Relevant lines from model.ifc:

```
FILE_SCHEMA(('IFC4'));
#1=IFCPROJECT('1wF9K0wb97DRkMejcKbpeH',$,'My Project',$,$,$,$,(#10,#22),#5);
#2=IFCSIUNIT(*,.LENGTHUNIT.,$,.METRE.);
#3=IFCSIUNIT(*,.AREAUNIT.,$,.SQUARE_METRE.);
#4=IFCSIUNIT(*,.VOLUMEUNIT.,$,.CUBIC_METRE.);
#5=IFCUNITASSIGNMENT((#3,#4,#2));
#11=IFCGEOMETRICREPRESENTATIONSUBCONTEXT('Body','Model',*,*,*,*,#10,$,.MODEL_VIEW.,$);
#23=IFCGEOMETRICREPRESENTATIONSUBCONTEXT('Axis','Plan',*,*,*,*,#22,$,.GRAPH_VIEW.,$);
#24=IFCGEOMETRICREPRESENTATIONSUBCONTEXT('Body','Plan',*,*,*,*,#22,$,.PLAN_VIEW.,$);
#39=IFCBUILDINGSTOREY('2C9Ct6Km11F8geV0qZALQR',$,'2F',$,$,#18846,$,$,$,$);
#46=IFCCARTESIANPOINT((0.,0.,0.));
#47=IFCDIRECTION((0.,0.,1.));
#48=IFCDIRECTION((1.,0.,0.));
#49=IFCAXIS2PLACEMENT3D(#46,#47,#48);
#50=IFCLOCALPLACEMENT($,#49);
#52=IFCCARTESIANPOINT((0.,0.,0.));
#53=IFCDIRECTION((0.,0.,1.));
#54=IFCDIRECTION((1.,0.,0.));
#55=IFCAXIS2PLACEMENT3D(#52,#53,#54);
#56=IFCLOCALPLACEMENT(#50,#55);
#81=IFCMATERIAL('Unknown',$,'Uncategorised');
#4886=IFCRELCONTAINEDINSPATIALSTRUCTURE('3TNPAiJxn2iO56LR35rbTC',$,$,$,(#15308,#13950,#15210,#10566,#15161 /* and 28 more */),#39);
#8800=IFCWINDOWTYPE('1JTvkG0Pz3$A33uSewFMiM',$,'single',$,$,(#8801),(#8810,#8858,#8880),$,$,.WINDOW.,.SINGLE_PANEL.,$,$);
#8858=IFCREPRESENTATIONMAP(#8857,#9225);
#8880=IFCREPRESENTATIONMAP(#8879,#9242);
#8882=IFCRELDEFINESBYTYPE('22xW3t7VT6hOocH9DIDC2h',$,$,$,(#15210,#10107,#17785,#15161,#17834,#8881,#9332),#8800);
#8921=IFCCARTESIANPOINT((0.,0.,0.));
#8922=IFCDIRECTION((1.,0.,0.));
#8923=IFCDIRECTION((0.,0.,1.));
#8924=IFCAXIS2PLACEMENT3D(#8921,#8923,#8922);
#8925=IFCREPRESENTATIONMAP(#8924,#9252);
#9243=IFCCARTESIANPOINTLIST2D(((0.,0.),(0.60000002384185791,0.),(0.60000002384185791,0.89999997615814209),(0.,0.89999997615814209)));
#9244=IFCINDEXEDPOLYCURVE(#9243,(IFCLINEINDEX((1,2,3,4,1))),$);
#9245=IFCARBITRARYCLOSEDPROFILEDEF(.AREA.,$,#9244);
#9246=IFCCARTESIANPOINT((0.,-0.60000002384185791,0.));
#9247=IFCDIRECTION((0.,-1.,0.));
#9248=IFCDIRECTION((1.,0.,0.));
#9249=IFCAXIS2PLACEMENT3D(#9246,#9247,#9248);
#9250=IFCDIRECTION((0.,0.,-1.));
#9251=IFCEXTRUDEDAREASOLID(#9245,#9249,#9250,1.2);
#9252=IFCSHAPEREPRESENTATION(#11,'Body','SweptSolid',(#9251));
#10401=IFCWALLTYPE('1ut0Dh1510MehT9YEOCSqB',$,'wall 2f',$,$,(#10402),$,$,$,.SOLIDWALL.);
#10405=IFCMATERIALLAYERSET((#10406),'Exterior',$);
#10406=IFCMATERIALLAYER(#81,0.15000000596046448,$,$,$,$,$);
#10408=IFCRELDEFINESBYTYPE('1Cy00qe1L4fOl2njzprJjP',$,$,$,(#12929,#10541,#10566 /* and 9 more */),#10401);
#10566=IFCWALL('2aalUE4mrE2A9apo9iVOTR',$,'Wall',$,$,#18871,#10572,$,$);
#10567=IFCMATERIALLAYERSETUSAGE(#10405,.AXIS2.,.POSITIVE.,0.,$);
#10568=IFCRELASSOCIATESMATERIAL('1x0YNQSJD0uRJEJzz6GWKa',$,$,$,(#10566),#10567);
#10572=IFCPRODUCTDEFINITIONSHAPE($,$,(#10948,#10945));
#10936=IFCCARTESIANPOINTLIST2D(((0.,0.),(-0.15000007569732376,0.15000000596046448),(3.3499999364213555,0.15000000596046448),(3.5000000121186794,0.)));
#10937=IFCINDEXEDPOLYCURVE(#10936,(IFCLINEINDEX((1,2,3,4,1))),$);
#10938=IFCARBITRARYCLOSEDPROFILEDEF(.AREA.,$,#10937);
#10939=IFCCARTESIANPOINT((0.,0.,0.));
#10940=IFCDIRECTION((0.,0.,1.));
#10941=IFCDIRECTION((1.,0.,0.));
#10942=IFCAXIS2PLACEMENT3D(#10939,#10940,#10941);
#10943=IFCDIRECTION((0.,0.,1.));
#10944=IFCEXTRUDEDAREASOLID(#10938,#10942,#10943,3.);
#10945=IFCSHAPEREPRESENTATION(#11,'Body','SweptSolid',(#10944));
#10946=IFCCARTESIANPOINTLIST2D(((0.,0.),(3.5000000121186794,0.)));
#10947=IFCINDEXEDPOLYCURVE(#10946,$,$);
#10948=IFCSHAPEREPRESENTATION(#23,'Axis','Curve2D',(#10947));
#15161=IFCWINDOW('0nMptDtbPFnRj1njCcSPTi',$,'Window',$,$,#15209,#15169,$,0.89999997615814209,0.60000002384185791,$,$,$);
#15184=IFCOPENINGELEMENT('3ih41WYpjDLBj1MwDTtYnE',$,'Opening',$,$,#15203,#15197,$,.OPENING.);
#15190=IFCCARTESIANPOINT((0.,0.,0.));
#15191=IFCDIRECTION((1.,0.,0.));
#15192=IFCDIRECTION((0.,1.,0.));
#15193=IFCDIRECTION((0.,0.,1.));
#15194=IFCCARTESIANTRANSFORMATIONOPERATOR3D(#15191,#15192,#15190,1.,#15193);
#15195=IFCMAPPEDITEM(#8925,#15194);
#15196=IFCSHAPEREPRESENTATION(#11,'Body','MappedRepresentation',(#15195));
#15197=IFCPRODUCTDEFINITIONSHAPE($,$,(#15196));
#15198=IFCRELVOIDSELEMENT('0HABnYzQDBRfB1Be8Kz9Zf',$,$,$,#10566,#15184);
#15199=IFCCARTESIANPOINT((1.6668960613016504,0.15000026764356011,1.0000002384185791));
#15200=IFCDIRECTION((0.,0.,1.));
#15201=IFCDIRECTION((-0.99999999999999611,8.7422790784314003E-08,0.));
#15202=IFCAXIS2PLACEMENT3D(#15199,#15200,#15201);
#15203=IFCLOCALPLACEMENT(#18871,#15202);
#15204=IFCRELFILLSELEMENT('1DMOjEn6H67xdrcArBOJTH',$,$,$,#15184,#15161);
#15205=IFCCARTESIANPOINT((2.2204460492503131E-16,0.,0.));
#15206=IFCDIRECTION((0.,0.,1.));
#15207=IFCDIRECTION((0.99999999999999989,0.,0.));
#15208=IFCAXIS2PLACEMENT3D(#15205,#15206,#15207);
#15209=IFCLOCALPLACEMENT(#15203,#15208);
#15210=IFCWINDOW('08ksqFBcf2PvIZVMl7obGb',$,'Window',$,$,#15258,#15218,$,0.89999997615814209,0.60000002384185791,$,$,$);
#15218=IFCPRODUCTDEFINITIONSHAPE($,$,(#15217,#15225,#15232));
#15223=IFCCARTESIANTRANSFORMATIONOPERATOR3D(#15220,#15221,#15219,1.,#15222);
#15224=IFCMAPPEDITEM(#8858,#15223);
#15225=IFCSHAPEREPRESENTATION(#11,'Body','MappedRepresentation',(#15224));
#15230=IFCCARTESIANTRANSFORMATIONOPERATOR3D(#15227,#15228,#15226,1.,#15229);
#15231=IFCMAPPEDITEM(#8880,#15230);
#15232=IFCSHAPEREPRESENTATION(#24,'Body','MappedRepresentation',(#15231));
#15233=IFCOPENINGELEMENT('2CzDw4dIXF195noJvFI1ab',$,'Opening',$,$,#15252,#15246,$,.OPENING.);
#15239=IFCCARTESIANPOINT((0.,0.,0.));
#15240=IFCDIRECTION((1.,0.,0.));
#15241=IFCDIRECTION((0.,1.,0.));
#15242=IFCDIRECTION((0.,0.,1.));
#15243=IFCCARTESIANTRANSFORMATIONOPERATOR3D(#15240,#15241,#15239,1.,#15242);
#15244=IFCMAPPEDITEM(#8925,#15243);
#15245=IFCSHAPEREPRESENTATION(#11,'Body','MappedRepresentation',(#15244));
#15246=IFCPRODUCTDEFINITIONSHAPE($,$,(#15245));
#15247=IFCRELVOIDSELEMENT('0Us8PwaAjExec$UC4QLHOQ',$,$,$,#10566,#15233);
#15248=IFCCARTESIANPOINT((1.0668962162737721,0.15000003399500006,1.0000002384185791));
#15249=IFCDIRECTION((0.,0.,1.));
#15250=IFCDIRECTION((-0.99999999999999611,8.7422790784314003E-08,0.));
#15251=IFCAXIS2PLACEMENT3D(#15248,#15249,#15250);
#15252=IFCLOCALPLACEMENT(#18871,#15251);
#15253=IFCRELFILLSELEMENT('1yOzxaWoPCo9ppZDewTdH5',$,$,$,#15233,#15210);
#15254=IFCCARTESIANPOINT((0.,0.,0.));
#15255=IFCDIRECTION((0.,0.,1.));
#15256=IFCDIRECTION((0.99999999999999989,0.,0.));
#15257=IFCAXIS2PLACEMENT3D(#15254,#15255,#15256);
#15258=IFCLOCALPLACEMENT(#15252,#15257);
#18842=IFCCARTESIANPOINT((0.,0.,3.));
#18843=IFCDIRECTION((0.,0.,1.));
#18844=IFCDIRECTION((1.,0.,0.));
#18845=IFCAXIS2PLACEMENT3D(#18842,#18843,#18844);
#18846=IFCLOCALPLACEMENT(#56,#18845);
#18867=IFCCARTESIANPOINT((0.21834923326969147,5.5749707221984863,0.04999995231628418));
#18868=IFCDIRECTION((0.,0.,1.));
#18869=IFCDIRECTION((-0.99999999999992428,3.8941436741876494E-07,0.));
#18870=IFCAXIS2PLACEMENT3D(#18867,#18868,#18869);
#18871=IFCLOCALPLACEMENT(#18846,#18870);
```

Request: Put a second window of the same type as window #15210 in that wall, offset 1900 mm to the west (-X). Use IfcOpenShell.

```python
import ifcopenshell
import ifcopenshell.api.feature
import ifcopenshell.api.geometry
import ifcopenshell.api.root
import ifcopenshell.geom
import ifcopenshell.util.element
import ifcopenshell.util.placement
import ifcopenshell.util.shape
import ifcopenshell.util.unit

model = ifcopenshell.open("model.ifc")
unit_scale = ifcopenshell.util.unit.calculate_unit_scale(model)
settings = ifcopenshell.geom.settings()


def volume(element):
    """Net volume in cubic metres, openings subtracted."""
    shape = ifcopenshell.geom.create_shape(settings, element)
    return ifcopenshell.util.shape.get_volume(shape.geometry)


window = model.by_guid("08ksqFBcf2PvIZVMl7obGb")
opening = window.FillsVoids[0].RelatingOpeningElement
wall = opening.VoidsElements[0].RelatingBuildingElement
before = volume(wall)
shift = ifcopenshell.util.placement.get_local_placement(wall.ObjectPlacement)[:3, 0] * 1.9 / unit_scale

# copy_class copies the void relationship, type, container and properties, but no geometry.
new_opening = ifcopenshell.api.root.copy_class(model, product=opening)
new_opening.Representation = ifcopenshell.util.element.copy_deep(
    model, opening.Representation, exclude=["IfcGeometricRepresentationContext", "IfcRepresentationMap"]
)
new_window = ifcopenshell.api.root.copy_class(model, product=window)
new_window.Representation = ifcopenshell.util.element.copy_deep(
    model, window.Representation, exclude=["IfcGeometricRepresentationContext", "IfcRepresentationMap"]
)
ifcopenshell.api.feature.add_filling(model, opening=new_opening, element=new_window)

for old, new in ((opening, new_opening), (window, new_window)):
    matrix = ifcopenshell.util.placement.get_local_placement(old.ObjectPlacement)
    matrix[:3, 3] += shift
    ifcopenshell.api.geometry.edit_object_placement(model, product=new, matrix=matrix, is_si=False)

after = volume(wall)

print(f"wall volume {before:.3f} -> {after:.3f} m3")

model.write("model-out.ifc")
```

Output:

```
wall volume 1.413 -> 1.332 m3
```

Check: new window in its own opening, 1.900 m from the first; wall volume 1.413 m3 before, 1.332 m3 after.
